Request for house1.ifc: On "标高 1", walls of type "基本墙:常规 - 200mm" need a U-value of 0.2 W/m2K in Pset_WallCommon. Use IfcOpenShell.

First a look at what the model holds.

```python
import ifcopenshell
import ifcopenshell.util.element

model = ifcopenshell.open("house1.ifc")
print(model.schema)
storey = next(s for s in model.by_type("IfcBuildingStorey") if s.Name == "标高 1")
walls = [e for e in ifcopenshell.util.element.get_decomposition(storey) if e.is_a("IfcWall")]
seen = {}
for e in walls:
    element_type = ifcopenshell.util.element.get_type(e)
    key = (element_type.Name if element_type != e and element_type else None, ifcopenshell.util.element.get_pset(e, "Pset_WallCommon", "ThermalTransmittance"))
    seen[key] = seen.get(key, 0) + 1
for (name, value), count in sorted(seen.items(), key=str):
    print(count, "x", name, "|", value)
```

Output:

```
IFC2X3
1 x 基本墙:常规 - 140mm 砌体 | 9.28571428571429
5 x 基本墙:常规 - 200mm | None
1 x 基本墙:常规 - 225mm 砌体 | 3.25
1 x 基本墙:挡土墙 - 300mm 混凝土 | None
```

```python
import ifcopenshell
import ifcopenshell.api.pset
import ifcopenshell.util.element

model = ifcopenshell.open("house1.ifc")

storey = next(s for s in model.by_type("IfcBuildingStorey") if s.Name == "标高 1")
walls = [e for e in ifcopenshell.util.element.get_decomposition(storey) if e.is_a("IfcWall")]

count = 0
for e in walls:
    element_type = ifcopenshell.util.element.get_type(e)
    if element_type in (None, e) or element_type.Name != "基本墙:常规 - 200mm":
        continue
    # add_pset returns the element's existing set when there is one.
    pset = ifcopenshell.api.pset.add_pset(model, product=e, name="Pset_WallCommon")
    ifcopenshell.api.pset.edit_pset(model, pset=pset, properties={"ThermalTransmittance": 0.2})
    count += 1

print(count, "walls updated")

model.write("house1-out.ifc")
```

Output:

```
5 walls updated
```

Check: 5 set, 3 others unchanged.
